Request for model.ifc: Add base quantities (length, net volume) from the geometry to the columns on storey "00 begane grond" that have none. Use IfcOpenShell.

First a look at what the model holds.

```python
import ifcopenshell
import ifcopenshell.util.element
import ifcopenshell.util.unit

model = ifcopenshell.open("model.ifc")
print(model.schema)
for unit_type in ("LENGTHUNIT", "AREAUNIT", "VOLUMEUNIT"):
    print(unit_type, ifcopenshell.util.unit.calculate_unit_scale(model, unit_type))
storey = next(s for s in model.by_type("IfcBuildingStorey") if s.Name == "00 begane grond")
columns = [e for e in ifcopenshell.util.element.get_decomposition(storey) if e.is_a("IfcColumn")]
for e in sorted(columns, key=lambda e: e.id()):
    print(e.id(), e.is_a(), e.Name, list(ifcopenshell.util.element.get_psets(e, qtos_only=True)), sep=" | ")
```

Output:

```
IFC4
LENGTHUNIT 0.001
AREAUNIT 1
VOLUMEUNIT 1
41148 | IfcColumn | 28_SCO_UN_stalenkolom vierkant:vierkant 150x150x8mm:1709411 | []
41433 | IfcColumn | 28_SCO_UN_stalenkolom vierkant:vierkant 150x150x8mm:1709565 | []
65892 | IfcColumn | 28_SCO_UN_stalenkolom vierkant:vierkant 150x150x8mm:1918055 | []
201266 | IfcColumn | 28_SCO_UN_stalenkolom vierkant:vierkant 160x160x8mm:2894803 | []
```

```python
import ifcopenshell
import ifcopenshell.api.pset
import ifcopenshell.geom
import ifcopenshell.util.element
import ifcopenshell.util.shape
import ifcopenshell.util.unit

model = ifcopenshell.open("model.ifc")
unit_scale = ifcopenshell.util.unit.calculate_unit_scale(model)
volume_scale = ifcopenshell.util.unit.calculate_unit_scale(model, "VOLUMEUNIT")
settings = ifcopenshell.geom.settings()

storey = next(s for s in model.by_type("IfcBuildingStorey") if s.Name == "00 begane grond")
columns = [e for e in ifcopenshell.util.element.get_decomposition(storey) if e.is_a("IfcColumn")]

for e in sorted(columns, key=lambda e: e.id()):
    if ifcopenshell.util.element.get_psets(e, qtos_only=True, should_inherit=False):
        continue
    # Geometry comes back in metres, in the element's own axes.
    shape = ifcopenshell.geom.create_shape(settings, e)
    values = {
        "Length": ifcopenshell.util.shape.get_z(shape.geometry) / unit_scale,
        "NetVolume": ifcopenshell.util.shape.get_volume(shape.geometry) / volume_scale,
    }
    qto = ifcopenshell.api.pset.add_qto(model, product=e, name="Qto_ColumnBaseQuantities")
    ifcopenshell.api.pset.edit_qto(model, qto=qto, properties=values)
    print(e.id(), {k: round(v, 3) for k, v in values.items()})

model.write("model-out.ifc")
```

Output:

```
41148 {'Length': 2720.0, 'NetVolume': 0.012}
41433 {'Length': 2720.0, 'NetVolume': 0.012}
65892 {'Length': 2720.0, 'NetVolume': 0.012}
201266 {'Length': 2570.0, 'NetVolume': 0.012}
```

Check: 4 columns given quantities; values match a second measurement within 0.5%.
